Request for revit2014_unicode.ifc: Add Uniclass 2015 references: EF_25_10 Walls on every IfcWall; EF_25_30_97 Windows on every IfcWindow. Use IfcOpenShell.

First a look at what the model holds.

```python
import ifcopenshell

model = ifcopenshell.open("revit2014_unicode.ifc")
print(model.schema)
print("classifications:", [c.Name for c in model.by_type("IfcClassification")])
for ifc_class in ("IfcDoor", "IfcRoof", "IfcStair", "IfcWall", "IfcWindow"):
    print(ifc_class, len(model.by_type(ifc_class)))
```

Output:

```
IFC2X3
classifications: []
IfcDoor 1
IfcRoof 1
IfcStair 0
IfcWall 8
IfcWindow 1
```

```python
import ifcopenshell
import ifcopenshell.api.classification

model = ifcopenshell.open("revit2014_unicode.ifc")

# IFC2X3 requires Source and Edition and has no link from the project to the system.
system = model.create_entity("IfcClassification", Source="NBS", Edition="2015", Name="Uniclass 2015")

codes = {
    "IfcWall": ("EF_25_10", "Walls"),
    "IfcWindow": ("EF_25_30_97", "Windows"),
}
for ifc_class, (code, name) in codes.items():
    products = model.by_type(ifc_class)
    ifcopenshell.api.classification.add_reference(
        model, products=products, classification=system, identification=code, name=name
    )
    print(code, len(products))

model.write("revit2014_unicode_edited.ifc")
```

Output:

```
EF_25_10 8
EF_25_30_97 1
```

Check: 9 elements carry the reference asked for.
